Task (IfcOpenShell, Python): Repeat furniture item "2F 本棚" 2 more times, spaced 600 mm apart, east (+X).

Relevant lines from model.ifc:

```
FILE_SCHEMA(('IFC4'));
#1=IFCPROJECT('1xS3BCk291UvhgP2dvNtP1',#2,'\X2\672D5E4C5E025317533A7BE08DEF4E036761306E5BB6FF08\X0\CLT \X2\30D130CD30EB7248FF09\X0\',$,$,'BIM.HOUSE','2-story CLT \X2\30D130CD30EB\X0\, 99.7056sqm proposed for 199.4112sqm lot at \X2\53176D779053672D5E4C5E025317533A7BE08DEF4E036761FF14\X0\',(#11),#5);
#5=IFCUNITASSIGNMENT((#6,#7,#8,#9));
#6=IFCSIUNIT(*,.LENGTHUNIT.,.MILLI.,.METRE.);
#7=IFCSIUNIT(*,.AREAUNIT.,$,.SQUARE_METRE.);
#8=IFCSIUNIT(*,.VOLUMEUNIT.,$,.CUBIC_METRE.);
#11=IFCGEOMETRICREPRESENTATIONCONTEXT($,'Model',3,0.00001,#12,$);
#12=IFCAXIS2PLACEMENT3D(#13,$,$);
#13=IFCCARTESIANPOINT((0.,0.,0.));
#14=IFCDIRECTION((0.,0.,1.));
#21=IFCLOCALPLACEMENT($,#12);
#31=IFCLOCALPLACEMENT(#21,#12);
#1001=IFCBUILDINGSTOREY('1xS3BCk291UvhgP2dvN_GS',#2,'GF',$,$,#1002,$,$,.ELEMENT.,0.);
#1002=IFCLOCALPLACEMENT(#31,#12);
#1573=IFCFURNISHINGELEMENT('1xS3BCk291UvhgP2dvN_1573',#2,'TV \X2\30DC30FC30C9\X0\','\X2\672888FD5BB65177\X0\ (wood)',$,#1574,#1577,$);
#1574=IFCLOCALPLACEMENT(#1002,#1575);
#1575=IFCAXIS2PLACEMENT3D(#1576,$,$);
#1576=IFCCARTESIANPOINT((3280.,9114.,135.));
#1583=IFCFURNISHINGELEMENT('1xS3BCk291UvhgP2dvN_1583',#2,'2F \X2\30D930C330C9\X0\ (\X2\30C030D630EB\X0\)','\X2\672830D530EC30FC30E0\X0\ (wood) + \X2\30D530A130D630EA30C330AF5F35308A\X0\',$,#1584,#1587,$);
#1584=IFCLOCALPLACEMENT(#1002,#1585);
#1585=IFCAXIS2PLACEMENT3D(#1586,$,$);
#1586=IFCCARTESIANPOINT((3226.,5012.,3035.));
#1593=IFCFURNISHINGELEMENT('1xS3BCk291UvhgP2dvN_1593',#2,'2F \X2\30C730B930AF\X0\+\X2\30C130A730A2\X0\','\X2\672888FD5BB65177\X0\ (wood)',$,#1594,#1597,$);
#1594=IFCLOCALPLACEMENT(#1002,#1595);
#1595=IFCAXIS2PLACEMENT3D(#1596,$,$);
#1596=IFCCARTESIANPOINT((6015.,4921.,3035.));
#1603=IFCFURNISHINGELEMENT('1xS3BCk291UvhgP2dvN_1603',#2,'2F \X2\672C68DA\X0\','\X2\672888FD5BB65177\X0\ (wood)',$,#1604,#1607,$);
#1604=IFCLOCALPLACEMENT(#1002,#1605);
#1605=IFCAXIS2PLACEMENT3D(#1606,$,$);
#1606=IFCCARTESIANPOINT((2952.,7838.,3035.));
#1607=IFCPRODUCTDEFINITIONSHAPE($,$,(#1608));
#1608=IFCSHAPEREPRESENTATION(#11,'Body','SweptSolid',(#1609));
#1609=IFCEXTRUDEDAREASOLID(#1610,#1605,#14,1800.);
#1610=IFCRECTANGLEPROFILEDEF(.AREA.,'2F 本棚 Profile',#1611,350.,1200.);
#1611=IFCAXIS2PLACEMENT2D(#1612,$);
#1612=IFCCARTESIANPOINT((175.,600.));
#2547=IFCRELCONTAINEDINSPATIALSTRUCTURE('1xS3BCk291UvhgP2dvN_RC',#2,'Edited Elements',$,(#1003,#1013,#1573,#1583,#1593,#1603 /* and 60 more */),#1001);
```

```python
import numpy as np
import ifcopenshell
import ifcopenshell.api.geometry
import ifcopenshell.api.root
import ifcopenshell.util.element
import ifcopenshell.util.placement

model = ifcopenshell.open("model.ifc")


def reuse_history(source, copy):
    """copy_class also copies each property set's owner history, people and application; keep the originals."""
    for rel in copy.IsDefinedBy:
        if rel.is_a("IfcRelDefinesByProperties") and (history := rel.RelatingPropertyDefinition.OwnerHistory):
            rel.RelatingPropertyDefinition.OwnerHistory = source.OwnerHistory
            ifcopenshell.util.element.remove_deep2(model, history)


source = model.by_guid("1xS3BCk291UvhgP2dvN_1603")
base = ifcopenshell.util.placement.get_local_placement(source.ObjectPlacement)
step = np.array([1.0, 0.0, 0.0]) * 600.0

for i in range(1, 3):
    copy = ifcopenshell.api.root.copy_class(model, product=source)
    copy.Representation = ifcopenshell.util.element.copy_deep(
        model, source.Representation, exclude=["IfcGeometricRepresentationContext", "IfcRepresentationMap"]
    )
    reuse_history(source, copy)
    matrix = base.copy()
    matrix[:3, 3] += i * step
    print("added at", matrix[:3, 3].round(3) + 0.0)
    ifcopenshell.api.geometry.edit_object_placement(model, product=copy, matrix=matrix, is_si=False)

model.write("model-out.ifc")
```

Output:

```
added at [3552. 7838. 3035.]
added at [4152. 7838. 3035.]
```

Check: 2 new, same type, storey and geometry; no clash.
